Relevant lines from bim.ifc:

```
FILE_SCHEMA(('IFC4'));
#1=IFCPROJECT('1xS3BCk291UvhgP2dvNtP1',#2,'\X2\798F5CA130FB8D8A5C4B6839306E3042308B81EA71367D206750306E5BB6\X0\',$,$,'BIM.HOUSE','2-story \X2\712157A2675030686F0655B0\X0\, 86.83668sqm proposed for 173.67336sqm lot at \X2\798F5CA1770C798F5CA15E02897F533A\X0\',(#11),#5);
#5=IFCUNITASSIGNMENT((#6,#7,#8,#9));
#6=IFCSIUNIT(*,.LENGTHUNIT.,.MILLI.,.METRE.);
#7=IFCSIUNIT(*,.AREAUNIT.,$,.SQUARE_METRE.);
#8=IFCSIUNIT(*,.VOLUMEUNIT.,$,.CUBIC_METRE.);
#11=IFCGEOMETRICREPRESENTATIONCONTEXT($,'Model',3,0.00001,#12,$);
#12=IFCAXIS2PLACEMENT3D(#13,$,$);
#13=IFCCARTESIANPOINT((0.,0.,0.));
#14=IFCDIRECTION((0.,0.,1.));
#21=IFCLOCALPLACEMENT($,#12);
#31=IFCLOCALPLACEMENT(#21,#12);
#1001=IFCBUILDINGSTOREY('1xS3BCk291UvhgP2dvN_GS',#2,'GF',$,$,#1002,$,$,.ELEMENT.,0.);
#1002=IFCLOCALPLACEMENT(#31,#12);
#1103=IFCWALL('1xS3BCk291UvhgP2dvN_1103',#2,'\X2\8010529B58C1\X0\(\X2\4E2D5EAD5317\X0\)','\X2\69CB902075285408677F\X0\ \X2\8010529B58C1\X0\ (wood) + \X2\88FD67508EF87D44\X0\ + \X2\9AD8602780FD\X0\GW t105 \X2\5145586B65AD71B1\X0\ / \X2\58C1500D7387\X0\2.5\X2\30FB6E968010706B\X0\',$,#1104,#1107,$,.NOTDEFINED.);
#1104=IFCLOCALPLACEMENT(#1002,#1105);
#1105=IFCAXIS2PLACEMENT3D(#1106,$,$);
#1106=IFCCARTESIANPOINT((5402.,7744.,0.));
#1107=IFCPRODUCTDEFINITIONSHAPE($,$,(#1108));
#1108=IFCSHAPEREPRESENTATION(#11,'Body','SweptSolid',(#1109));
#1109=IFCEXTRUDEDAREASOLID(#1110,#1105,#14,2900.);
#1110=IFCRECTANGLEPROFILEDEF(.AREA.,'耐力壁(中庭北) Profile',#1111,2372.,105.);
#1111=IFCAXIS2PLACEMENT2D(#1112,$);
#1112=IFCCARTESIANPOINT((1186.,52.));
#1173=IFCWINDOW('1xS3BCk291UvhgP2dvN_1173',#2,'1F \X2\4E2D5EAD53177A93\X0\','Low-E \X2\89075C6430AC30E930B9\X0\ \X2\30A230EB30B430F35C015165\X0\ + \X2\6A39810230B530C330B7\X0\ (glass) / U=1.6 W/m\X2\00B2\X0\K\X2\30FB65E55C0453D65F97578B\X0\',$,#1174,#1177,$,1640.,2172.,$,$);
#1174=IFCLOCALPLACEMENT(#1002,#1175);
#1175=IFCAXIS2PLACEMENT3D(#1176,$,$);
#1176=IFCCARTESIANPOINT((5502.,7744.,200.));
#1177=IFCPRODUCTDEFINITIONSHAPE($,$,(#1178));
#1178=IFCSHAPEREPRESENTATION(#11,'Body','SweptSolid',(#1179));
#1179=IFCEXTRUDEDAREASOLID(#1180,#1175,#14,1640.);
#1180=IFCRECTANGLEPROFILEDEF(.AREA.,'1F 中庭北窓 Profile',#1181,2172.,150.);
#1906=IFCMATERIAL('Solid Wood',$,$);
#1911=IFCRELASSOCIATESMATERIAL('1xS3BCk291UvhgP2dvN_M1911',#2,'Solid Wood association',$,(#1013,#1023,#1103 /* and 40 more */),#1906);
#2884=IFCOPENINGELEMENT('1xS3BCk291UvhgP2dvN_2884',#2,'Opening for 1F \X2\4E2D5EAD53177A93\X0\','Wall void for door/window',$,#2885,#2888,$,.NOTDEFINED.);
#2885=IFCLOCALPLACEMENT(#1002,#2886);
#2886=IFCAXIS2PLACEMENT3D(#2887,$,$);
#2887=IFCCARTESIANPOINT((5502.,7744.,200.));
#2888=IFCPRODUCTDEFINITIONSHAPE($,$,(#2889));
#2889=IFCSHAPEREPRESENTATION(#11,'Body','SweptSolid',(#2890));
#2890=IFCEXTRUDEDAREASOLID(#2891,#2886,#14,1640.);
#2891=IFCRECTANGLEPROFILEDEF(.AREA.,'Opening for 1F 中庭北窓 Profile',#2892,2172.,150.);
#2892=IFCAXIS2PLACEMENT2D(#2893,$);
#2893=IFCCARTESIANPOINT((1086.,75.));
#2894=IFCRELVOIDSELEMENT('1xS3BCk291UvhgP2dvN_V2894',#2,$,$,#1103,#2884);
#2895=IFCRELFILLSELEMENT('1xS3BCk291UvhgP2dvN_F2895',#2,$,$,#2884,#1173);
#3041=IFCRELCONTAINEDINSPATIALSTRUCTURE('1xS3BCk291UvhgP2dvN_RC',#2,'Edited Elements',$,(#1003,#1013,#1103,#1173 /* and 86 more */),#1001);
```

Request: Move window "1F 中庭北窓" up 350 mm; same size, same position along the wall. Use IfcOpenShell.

```python
import numpy as np
import ifcopenshell
import ifcopenshell.api.geometry
import ifcopenshell.util.placement
import ifcopenshell.util.unit

model = ifcopenshell.open("bim.ifc")
unit_scale = ifcopenshell.util.unit.calculate_unit_scale(model)

window = model.by_guid("1xS3BCk291UvhgP2dvN_1173")
opening = window.FillsVoids[0].RelatingOpeningElement
dz = 350.0

shift = np.array([0.0, 0.0, dz])
# The window is not placed relative to its opening, so move both.
for product in (opening, window):
    matrix = ifcopenshell.util.placement.get_local_placement(product.ObjectPlacement)
    matrix[:3, 3] += shift
    ifcopenshell.api.geometry.edit_object_placement(model, product=product, matrix=matrix, is_si=False)

print(f"moved by {dz * unit_scale:+.3f} m")

model.write("bim_v2.ifc")
```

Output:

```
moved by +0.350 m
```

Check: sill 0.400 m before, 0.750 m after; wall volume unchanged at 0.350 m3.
